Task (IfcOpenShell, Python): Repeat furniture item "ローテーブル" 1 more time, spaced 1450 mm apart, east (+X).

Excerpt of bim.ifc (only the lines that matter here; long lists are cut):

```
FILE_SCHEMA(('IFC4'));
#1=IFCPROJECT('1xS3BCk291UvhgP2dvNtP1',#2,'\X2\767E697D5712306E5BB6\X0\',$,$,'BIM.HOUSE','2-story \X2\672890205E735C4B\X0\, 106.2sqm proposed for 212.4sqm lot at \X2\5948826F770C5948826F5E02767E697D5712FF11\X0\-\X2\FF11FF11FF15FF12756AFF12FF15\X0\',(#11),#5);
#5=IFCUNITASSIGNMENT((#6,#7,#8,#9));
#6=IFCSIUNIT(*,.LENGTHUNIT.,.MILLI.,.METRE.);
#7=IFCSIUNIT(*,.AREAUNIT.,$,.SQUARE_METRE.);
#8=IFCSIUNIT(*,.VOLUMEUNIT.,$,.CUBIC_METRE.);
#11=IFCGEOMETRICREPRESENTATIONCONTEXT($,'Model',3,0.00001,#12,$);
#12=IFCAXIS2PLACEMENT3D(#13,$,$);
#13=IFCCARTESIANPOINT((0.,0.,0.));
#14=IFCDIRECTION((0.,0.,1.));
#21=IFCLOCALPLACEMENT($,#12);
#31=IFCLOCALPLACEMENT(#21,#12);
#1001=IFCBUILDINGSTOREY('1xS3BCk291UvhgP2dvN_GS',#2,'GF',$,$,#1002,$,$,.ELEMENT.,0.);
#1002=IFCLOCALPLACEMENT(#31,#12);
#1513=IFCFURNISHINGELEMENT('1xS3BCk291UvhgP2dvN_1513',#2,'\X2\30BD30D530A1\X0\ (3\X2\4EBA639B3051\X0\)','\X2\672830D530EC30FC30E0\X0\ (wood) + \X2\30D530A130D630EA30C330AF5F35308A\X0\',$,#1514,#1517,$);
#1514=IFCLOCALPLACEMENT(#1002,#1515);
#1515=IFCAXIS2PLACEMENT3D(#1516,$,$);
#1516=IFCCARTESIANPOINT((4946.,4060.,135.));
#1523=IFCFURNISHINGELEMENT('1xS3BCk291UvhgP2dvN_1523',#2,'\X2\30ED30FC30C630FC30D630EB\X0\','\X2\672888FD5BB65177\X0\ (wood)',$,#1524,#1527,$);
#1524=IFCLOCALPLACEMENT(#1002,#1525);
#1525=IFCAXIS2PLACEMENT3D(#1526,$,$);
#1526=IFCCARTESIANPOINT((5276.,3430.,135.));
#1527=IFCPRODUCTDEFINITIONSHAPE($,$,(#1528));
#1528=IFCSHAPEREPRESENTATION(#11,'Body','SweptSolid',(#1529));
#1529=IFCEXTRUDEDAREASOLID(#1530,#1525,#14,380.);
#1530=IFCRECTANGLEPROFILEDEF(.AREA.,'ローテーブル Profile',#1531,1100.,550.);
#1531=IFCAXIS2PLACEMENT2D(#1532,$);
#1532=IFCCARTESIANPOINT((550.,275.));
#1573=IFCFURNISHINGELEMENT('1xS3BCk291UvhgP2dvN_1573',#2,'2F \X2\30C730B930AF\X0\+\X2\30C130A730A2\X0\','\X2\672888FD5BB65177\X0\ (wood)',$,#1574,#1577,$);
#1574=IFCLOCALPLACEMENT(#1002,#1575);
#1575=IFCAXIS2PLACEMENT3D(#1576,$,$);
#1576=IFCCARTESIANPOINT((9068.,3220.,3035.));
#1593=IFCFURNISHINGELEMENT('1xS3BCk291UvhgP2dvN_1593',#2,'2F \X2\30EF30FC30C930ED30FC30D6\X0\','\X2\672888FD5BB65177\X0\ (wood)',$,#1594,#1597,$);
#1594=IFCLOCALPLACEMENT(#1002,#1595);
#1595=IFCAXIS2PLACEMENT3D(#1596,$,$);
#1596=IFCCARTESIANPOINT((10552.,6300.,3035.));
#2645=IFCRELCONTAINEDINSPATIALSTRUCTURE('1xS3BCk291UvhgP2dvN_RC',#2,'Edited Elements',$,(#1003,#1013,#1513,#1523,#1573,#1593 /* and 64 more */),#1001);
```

```python
import numpy as np
import ifcopenshell
import ifcopenshell.api.geometry
import ifcopenshell.api.root
import ifcopenshell.util.element
import ifcopenshell.util.placement
import ifcopenshell.util.unit

model = ifcopenshell.open("bim.ifc")
unit_scale = ifcopenshell.util.unit.calculate_unit_scale(model)


def reuse_history(source, copy):
    """copy_class also copies each property set's owner history, people and application; keep the originals."""
    for rel in copy.IsDefinedBy:
        if rel.is_a("IfcRelDefinesByProperties") and (history := rel.RelatingPropertyDefinition.OwnerHistory):
            rel.RelatingPropertyDefinition.OwnerHistory = source.OwnerHistory
            ifcopenshell.util.element.remove_deep2(model, history)


source = model.by_guid("1xS3BCk291UvhgP2dvN_1523")
base = ifcopenshell.util.placement.get_local_placement(source.ObjectPlacement)
step = np.array([1.0, 0.0, 0.0]) * 1.45 / unit_scale

for i in range(1, 2):
    copy = ifcopenshell.api.root.copy_class(model, product=source)
    copy.Representation = ifcopenshell.util.element.copy_deep(
        model, source.Representation, exclude=["IfcGeometricRepresentationContext", "IfcRepresentationMap"]
    )
    reuse_history(source, copy)
    matrix = base.copy()
    matrix[:3, 3] += i * step
    print("added at", matrix[:3, 3].round(3) + 0.0)
    ifcopenshell.api.geometry.edit_object_placement(model, product=copy, matrix=matrix, is_si=False)

model.write("bim_rev.ifc")
```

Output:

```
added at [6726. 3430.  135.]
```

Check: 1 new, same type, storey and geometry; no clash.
